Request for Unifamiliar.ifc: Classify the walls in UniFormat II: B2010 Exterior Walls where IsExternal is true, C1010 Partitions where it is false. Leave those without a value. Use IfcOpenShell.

First a look at what the model holds.

```python
import ifcopenshell
import ifcopenshell.util.element

model = ifcopenshell.open("Unifamiliar.ifc")
print(model.schema)
print("classifications:", [c.Name for c in model.by_type("IfcClassification")])
values = [ifcopenshell.util.element.get_pset(e, "Pset_WallCommon", "IsExternal") for e in model.by_type("IfcWall")]
for value in (True, False, None):
    print("IsExternal", value, values.count(value))
```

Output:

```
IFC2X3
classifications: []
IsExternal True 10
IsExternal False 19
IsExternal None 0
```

```python
import ifcopenshell
import ifcopenshell.api.classification
import ifcopenshell.util.element

model = ifcopenshell.open("Unifamiliar.ifc")

# IFC2X3 requires Source and Edition and has no link from the project to the system.
system = model.create_entity("IfcClassification", Source="ASTM", Edition="E1557", Name="UniFormat II")

walls = model.by_type("IfcWall")
external = {e: ifcopenshell.util.element.get_pset(e, "Pset_WallCommon", "IsExternal") for e in walls}
for flag, code, name in ((True, "B2010", "Exterior Walls"), (False, "C1010", "Partitions")):
    products = [e for e in walls if external[e] is flag]
    ifcopenshell.api.classification.add_reference(
        model, products=products, classification=system, identification=code, name=name
    )
    print(code, len(products))

model.write("Unifamiliar_edited.ifc")
```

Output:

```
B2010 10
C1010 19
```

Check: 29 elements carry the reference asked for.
